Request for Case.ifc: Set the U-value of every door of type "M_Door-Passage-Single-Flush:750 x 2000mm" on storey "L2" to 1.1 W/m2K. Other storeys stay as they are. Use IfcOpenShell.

First a look at what the model holds.

```python
import ifcopenshell
import ifcopenshell.util.element

model = ifcopenshell.open("Case.ifc")
print(model.schema)
storey = next(s for s in model.by_type("IfcBuildingStorey") if s.Name == "L2")
doors = [e for e in ifcopenshell.util.element.get_decomposition(storey) if e.is_a("IfcDoor")]
seen = {}
for e in doors:
    element_type = ifcopenshell.util.element.get_type(e)
    key = (element_type.Name if element_type != e and element_type else None, ifcopenshell.util.element.get_pset(e, "Pset_DoorCommon", "ThermalTransmittance"))
    seen[key] = seen.get(key, 0) + 1
for (name, value), count in sorted(seen.items(), key=str):
    print(count, "x", name, "|", value)
```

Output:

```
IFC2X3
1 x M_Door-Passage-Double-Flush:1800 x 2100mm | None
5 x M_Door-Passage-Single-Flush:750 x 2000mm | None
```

```python
import ifcopenshell
import ifcopenshell.api.pset
import ifcopenshell.util.element

model = ifcopenshell.open("Case.ifc")

storey = next(s for s in model.by_type("IfcBuildingStorey") if s.Name == "L2")
doors = [e for e in ifcopenshell.util.element.get_decomposition(storey) if e.is_a("IfcDoor")]

count = 0
for e in doors:
    element_type = ifcopenshell.util.element.get_type(e)
    if element_type in (None, e) or element_type.Name != "M_Door-Passage-Single-Flush:750 x 2000mm":
        continue
    # add_pset returns the element's existing set when there is one.
    pset = ifcopenshell.api.pset.add_pset(model, product=e, name="Pset_DoorCommon")
    ifcopenshell.api.pset.edit_pset(model, pset=pset, properties={"ThermalTransmittance": 1.1})
    count += 1

print(count, "doors updated")

model.write("Case_updated.ifc")
```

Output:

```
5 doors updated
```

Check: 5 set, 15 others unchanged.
